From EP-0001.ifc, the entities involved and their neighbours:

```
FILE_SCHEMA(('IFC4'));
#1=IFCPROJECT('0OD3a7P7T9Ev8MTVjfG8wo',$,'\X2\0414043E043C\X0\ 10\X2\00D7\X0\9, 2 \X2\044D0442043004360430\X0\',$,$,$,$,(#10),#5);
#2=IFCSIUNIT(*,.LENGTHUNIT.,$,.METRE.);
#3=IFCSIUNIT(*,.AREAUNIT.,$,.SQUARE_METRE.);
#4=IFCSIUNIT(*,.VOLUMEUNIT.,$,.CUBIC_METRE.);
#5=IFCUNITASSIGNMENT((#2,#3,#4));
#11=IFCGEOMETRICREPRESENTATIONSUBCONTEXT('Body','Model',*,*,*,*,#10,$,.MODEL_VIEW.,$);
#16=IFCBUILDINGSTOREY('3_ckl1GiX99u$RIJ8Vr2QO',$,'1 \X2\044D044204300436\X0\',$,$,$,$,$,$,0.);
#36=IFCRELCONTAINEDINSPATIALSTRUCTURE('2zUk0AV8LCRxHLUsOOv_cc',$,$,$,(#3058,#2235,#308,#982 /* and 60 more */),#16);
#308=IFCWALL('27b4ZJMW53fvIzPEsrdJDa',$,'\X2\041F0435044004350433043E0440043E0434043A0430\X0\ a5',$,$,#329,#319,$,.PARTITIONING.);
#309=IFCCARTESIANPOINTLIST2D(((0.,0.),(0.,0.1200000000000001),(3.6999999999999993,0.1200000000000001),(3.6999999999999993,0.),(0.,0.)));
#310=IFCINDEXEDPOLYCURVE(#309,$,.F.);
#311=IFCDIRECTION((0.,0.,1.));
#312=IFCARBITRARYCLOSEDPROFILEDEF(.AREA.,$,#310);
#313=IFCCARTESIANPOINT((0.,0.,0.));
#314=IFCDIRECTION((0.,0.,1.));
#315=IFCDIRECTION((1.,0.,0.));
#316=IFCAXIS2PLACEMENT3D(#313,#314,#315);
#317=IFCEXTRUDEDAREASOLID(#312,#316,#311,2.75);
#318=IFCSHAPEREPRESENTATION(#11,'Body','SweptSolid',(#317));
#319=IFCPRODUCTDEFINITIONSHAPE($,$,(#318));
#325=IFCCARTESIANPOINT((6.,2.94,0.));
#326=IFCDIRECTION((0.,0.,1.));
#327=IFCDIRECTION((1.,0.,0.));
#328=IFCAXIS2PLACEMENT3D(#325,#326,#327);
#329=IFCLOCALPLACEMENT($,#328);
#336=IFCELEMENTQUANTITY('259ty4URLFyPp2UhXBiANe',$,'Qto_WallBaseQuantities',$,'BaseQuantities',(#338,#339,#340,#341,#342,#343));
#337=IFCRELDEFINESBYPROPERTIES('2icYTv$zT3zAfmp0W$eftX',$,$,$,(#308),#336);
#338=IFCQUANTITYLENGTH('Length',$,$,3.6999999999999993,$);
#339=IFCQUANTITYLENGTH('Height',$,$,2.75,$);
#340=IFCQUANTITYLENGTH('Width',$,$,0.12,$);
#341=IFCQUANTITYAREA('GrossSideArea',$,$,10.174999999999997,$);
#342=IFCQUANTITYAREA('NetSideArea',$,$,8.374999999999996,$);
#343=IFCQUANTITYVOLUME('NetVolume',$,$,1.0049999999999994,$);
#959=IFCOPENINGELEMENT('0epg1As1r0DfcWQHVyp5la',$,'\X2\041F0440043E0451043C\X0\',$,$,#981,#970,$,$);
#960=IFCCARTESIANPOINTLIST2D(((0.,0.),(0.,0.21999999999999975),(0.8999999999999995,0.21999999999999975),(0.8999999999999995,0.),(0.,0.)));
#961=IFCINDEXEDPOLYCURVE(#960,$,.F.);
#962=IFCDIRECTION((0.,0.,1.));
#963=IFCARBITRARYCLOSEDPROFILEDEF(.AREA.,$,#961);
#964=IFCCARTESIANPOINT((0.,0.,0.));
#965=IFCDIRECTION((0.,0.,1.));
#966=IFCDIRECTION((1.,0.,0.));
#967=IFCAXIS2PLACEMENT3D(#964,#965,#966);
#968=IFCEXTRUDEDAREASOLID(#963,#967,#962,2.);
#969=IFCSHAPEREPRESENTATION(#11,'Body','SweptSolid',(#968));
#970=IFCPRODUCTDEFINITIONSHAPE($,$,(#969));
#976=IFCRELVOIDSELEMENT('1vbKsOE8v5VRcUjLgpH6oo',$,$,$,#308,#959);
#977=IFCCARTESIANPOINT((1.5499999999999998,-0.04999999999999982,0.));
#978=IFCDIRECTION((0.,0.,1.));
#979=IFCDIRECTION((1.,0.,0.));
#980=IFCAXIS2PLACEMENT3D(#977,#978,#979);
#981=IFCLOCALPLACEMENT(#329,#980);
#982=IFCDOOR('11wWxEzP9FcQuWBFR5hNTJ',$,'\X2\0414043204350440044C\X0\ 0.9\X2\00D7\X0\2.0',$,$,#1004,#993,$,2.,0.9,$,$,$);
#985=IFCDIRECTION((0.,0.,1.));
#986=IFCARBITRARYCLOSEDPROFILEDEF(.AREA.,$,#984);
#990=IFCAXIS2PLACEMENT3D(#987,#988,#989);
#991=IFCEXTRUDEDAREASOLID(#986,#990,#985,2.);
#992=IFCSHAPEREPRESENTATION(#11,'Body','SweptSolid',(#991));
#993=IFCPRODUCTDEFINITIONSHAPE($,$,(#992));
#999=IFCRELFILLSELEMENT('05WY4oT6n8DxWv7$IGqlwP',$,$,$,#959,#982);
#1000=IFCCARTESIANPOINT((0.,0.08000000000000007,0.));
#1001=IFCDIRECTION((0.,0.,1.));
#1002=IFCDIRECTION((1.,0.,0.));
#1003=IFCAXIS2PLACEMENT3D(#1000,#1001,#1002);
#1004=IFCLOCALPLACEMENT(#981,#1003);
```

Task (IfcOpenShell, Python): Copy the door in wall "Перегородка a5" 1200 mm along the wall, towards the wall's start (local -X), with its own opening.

```python
import ifcopenshell
import ifcopenshell.api.feature
import ifcopenshell.api.geometry
import ifcopenshell.api.pset
import ifcopenshell.api.root
import ifcopenshell.geom
import ifcopenshell.util.element
import ifcopenshell.util.placement
import ifcopenshell.util.shape
import ifcopenshell.util.unit

model = ifcopenshell.open("EP-0001.ifc")
unit_scale = ifcopenshell.util.unit.calculate_unit_scale(model)
area_scale = ifcopenshell.util.unit.calculate_unit_scale(model, "AREAUNIT")
volume_scale = ifcopenshell.util.unit.calculate_unit_scale(model, "VOLUMEUNIT")
settings = ifcopenshell.geom.settings()


def volume(element):
    """Net volume in cubic metres, openings subtracted."""
    shape = ifcopenshell.geom.create_shape(settings, element)
    return ifcopenshell.util.shape.get_volume(shape.geometry)


door = model.by_guid("11wWxEzP9FcQuWBFR5hNTJ")
opening = door.FillsVoids[0].RelatingOpeningElement
wall = opening.VoidsElements[0].RelatingBuildingElement
before = volume(wall)
shift = ifcopenshell.util.placement.get_local_placement(wall.ObjectPlacement)[:3, 0] * -1.2 / unit_scale

# copy_class copies the void relationship, type, container and properties, but no geometry.
new_opening = ifcopenshell.api.root.copy_class(model, product=opening)
new_opening.Representation = ifcopenshell.util.element.copy_deep(
    model, opening.Representation, exclude=["IfcGeometricRepresentationContext", "IfcRepresentationMap"]
)
new_door = ifcopenshell.api.root.copy_class(model, product=door)
new_door.Representation = ifcopenshell.util.element.copy_deep(
    model, door.Representation, exclude=["IfcGeometricRepresentationContext", "IfcRepresentationMap"]
)
ifcopenshell.api.feature.add_filling(model, opening=new_opening, element=new_door)

for old, new in ((opening, new_opening), (door, new_door)):
    matrix = ifcopenshell.util.placement.get_local_placement(old.ObjectPlacement)
    matrix[:3, 3] += shift
    ifcopenshell.api.geometry.edit_object_placement(model, product=new, matrix=matrix, is_si=False)

after = volume(wall)
thickness = 0.12  # wall thickness in metres

# Update the wall's stored quantities.
qto = model.by_id(ifcopenshell.util.element.get_pset(wall, "Qto_WallBaseQuantities", should_inherit=False)["id"])
ifcopenshell.api.pset.edit_qto(model, qto=qto, properties={
    "NetSideArea": after / thickness / area_scale,
    "NetVolume": after / volume_scale,
})

print(f"wall volume {before:.3f} -> {after:.3f} m3")

model.write("EP-0001-out.ifc")
```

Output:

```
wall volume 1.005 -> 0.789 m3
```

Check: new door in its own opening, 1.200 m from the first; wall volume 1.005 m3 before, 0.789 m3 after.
